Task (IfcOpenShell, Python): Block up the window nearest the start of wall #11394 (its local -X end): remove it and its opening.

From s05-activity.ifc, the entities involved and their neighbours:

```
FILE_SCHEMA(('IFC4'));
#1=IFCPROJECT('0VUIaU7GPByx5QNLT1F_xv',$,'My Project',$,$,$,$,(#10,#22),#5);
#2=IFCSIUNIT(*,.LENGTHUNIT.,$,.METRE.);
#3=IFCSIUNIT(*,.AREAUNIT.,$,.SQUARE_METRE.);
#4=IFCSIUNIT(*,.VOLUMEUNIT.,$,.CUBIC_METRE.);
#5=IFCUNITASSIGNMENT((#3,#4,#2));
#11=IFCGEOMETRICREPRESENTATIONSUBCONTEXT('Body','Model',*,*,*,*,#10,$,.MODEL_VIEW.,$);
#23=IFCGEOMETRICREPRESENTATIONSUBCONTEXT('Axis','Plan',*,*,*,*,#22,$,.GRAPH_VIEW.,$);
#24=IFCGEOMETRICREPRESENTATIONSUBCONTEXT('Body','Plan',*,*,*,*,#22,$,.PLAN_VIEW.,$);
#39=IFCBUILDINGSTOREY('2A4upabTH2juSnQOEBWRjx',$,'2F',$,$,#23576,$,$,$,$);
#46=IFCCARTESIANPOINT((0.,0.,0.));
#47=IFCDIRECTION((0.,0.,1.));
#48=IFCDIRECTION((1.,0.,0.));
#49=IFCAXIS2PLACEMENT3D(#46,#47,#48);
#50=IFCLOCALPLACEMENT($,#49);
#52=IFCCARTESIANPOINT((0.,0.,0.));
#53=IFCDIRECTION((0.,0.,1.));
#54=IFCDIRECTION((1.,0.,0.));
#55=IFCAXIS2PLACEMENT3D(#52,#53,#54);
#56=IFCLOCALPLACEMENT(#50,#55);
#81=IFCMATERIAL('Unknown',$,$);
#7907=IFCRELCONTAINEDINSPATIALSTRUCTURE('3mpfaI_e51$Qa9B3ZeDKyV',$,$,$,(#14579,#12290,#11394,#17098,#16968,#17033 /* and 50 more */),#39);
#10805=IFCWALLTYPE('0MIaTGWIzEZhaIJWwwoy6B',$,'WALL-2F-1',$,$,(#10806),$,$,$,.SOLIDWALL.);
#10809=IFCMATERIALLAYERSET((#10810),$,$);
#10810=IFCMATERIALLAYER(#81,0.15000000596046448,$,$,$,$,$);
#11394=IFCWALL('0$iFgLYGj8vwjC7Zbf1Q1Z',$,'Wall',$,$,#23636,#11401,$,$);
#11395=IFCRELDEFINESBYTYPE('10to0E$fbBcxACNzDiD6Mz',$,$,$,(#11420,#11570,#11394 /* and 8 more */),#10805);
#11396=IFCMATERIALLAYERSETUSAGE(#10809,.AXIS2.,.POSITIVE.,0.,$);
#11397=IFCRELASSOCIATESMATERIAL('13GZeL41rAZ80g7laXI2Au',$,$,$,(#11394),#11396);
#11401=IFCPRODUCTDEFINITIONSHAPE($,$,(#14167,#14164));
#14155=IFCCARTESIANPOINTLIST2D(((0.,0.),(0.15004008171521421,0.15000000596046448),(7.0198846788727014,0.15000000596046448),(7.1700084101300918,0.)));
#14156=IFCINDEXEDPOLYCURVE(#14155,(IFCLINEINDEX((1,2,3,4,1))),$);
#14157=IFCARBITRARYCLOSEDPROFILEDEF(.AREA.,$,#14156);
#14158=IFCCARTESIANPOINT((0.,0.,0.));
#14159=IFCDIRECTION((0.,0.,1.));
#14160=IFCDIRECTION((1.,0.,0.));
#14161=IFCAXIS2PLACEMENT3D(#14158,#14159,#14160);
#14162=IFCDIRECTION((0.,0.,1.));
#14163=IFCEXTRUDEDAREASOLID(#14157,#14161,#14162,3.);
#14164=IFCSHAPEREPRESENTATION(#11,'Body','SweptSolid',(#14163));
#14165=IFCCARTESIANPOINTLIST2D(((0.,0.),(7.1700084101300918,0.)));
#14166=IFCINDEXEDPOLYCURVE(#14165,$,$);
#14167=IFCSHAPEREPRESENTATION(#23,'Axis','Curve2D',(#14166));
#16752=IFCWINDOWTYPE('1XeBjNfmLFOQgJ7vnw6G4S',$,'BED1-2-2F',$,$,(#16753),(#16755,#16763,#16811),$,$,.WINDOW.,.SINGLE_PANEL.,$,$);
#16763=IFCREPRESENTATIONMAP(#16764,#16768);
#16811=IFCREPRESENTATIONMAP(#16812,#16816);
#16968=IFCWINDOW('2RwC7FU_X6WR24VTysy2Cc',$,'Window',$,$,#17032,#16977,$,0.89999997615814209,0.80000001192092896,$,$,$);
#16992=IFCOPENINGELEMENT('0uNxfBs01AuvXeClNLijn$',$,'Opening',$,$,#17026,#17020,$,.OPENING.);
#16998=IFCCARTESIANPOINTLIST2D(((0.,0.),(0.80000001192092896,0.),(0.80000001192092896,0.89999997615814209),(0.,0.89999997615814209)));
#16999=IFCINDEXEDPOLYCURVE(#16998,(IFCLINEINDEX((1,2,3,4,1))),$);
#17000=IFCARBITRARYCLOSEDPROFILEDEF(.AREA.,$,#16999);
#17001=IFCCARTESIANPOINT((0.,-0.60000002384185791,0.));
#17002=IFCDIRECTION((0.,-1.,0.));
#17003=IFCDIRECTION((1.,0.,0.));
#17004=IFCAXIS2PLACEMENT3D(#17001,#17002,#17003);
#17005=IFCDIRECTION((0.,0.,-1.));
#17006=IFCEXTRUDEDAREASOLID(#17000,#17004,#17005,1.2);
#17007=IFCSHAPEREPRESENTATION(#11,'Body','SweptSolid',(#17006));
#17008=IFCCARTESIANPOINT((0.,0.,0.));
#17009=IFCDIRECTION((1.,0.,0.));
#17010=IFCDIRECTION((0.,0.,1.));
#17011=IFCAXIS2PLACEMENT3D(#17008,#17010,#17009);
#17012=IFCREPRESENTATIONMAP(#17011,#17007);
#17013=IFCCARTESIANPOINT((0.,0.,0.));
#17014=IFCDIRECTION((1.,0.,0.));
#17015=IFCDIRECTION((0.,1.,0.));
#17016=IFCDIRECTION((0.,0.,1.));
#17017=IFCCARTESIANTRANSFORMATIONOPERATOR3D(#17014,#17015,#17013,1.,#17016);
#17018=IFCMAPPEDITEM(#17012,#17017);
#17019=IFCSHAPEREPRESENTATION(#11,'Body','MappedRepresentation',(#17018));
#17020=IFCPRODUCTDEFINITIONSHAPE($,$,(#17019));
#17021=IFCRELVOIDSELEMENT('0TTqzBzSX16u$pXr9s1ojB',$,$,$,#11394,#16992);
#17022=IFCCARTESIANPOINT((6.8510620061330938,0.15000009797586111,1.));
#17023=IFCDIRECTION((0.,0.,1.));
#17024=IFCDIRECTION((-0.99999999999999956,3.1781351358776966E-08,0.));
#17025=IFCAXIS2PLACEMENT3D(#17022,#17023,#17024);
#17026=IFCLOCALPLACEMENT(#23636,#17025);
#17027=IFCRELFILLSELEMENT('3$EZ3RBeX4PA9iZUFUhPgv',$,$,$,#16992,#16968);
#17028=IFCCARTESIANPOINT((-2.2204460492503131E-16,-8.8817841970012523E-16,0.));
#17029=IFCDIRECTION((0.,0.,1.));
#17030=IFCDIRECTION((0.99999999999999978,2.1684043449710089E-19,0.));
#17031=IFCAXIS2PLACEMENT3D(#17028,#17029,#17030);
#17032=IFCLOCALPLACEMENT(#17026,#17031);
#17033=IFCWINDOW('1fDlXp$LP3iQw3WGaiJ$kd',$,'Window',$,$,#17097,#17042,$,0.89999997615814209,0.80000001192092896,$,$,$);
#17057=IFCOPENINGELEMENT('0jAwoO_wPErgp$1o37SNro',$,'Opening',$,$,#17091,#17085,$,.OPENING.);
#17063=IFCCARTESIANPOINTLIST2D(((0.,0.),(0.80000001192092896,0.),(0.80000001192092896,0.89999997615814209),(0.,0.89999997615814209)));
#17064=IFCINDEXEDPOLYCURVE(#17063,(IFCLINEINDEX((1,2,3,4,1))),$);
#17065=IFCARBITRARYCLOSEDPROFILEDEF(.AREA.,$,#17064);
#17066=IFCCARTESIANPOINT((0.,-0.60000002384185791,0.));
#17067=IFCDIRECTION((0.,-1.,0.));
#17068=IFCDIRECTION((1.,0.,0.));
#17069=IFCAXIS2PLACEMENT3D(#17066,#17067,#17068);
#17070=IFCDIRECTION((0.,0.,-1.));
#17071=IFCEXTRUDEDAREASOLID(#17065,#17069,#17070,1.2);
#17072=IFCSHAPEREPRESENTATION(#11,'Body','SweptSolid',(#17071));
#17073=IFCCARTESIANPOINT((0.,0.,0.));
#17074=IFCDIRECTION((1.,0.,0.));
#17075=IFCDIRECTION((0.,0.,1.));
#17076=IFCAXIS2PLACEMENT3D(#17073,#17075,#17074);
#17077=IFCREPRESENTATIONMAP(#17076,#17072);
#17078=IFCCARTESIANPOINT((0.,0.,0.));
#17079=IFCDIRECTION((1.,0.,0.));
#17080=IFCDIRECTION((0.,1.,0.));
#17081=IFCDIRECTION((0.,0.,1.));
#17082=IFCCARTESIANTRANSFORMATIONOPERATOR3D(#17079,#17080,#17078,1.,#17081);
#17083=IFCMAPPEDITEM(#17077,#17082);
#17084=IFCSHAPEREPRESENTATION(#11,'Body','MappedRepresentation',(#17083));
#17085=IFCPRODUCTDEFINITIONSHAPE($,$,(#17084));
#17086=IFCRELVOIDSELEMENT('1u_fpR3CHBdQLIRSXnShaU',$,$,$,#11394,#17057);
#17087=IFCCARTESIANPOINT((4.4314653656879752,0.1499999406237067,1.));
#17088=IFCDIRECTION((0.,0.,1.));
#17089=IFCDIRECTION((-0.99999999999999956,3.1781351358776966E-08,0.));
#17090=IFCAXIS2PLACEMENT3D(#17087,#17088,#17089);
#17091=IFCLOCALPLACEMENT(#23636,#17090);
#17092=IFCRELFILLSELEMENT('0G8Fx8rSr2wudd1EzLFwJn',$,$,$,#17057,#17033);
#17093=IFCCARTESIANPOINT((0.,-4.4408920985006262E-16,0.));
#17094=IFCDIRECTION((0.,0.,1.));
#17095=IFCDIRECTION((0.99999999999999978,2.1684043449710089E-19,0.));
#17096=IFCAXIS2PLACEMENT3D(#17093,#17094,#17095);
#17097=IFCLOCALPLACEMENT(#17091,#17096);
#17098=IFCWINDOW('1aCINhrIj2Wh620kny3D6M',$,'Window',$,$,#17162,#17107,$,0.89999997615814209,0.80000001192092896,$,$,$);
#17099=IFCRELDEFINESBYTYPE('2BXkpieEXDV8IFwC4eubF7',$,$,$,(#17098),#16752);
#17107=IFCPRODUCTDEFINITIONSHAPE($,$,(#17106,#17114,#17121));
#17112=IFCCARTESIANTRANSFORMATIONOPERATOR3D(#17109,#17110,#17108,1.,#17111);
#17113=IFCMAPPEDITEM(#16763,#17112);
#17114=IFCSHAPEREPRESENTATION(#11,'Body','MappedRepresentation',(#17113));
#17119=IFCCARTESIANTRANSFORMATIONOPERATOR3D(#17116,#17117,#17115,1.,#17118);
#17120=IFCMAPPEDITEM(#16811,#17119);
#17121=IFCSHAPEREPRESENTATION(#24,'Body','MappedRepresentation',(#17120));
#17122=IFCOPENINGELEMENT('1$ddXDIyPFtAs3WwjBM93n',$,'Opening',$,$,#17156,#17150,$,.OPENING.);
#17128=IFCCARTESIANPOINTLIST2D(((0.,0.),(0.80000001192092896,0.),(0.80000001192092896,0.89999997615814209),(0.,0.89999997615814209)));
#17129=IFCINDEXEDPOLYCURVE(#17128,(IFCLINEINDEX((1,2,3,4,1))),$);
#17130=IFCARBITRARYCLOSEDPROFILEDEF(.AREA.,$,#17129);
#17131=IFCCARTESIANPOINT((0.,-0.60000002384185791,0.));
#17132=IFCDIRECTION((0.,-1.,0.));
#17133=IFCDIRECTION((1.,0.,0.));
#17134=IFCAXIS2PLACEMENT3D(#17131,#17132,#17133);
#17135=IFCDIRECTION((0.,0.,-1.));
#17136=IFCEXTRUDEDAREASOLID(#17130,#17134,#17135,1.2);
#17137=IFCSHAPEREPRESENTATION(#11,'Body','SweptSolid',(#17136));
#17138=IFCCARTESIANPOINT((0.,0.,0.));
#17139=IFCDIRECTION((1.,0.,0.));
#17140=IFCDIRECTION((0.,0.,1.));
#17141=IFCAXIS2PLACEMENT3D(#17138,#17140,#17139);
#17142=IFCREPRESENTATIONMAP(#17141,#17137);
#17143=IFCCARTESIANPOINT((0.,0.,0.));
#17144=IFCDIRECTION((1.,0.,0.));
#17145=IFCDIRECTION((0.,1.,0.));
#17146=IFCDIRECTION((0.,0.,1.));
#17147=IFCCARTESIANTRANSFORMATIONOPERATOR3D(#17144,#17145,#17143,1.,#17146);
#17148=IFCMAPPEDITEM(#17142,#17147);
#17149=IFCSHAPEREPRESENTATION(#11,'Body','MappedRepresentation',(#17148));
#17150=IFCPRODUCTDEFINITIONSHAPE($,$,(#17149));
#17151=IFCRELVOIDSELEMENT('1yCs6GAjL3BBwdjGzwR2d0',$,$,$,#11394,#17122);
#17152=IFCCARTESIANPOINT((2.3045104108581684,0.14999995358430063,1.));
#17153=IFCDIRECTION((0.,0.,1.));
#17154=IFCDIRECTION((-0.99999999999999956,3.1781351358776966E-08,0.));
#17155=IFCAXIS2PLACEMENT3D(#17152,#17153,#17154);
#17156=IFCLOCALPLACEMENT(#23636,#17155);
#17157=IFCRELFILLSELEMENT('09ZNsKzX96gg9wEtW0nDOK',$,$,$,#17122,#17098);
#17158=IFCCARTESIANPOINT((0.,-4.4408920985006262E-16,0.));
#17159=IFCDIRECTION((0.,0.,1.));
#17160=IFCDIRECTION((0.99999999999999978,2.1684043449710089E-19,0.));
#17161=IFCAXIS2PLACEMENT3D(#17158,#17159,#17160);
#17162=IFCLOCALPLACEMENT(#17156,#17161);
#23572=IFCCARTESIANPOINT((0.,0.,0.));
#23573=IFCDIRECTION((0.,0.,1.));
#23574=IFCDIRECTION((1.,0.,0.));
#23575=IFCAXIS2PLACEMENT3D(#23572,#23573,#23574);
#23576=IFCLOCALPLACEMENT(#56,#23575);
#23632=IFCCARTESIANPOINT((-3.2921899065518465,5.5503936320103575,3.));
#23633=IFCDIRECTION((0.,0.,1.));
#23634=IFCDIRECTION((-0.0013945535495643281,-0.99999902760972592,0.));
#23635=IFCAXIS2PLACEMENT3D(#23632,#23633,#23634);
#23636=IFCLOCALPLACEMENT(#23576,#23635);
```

```python
import ifcopenshell
import ifcopenshell.api.feature
import ifcopenshell.api.root
import ifcopenshell.geom
import ifcopenshell.util.shape

model = ifcopenshell.open("s05-activity.ifc")
settings = ifcopenshell.geom.settings()


def volume(element):
    """Net volume in cubic metres, openings subtracted."""
    shape = ifcopenshell.geom.create_shape(settings, element)
    return ifcopenshell.util.shape.get_volume(shape.geometry)


window = model.by_id(17098)
opening = window.FillsVoids[0].RelatingOpeningElement
wall = opening.VoidsElements[0].RelatingBuildingElement
before = volume(wall)

ifcopenshell.api.root.remove_product(model, product=window)
ifcopenshell.api.feature.remove_feature(model, feature=opening)

after = volume(wall)

print(f"wall volume {before:.3f} -> {after:.3f} m3")

model.write("s05-activity_edited.ifc")
```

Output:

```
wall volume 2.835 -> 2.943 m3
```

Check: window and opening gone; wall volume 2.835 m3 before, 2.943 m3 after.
